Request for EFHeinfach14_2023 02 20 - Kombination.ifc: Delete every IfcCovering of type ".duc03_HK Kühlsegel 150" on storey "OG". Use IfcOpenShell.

First a look at what the model holds.

```python
import ifcopenshell
import ifcopenshell.util.element

model = ifcopenshell.open("EFHeinfach14_2023 02 20 - Kombination.ifc")
print(model.schema)
storey = next(s for s in model.by_type("IfcBuildingStorey") if s.Name == "OG")
coverings = [e for e in ifcopenshell.util.element.get_decomposition(storey) if e.is_a("IfcCovering")]
seen = {}
for e in coverings:
    element_type = ifcopenshell.util.element.get_type(e)
    name = element_type.Name if element_type not in (None, e) else None
    seen[name] = seen.get(name, 0) + 1
for name, count in sorted(seen.items(), key=str):
    print(count, "x", name)
```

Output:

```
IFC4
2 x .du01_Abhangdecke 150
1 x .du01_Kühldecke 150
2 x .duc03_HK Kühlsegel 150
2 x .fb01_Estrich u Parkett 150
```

```python
import ifcopenshell
import ifcopenshell.api.root
import ifcopenshell.util.element

model = ifcopenshell.open("EFHeinfach14_2023 02 20 - Kombination.ifc")

storey = next(s for s in model.by_type("IfcBuildingStorey") if s.Name == "OG")
coverings = [e for e in ifcopenshell.util.element.get_decomposition(storey) if e.is_a("IfcCovering")]
targets = [e for e in coverings if (t := ifcopenshell.util.element.get_type(e)) not in (None, e) and t.Name == ".duc03_HK Kühlsegel 150"]

for e in targets:
    ifcopenshell.api.root.remove_product(model, product=e)
print(len(targets), "removed")

model.write("EFHeinfach14_2023 02 20 - Kombination_updated.ifc")
```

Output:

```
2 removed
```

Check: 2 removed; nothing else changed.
